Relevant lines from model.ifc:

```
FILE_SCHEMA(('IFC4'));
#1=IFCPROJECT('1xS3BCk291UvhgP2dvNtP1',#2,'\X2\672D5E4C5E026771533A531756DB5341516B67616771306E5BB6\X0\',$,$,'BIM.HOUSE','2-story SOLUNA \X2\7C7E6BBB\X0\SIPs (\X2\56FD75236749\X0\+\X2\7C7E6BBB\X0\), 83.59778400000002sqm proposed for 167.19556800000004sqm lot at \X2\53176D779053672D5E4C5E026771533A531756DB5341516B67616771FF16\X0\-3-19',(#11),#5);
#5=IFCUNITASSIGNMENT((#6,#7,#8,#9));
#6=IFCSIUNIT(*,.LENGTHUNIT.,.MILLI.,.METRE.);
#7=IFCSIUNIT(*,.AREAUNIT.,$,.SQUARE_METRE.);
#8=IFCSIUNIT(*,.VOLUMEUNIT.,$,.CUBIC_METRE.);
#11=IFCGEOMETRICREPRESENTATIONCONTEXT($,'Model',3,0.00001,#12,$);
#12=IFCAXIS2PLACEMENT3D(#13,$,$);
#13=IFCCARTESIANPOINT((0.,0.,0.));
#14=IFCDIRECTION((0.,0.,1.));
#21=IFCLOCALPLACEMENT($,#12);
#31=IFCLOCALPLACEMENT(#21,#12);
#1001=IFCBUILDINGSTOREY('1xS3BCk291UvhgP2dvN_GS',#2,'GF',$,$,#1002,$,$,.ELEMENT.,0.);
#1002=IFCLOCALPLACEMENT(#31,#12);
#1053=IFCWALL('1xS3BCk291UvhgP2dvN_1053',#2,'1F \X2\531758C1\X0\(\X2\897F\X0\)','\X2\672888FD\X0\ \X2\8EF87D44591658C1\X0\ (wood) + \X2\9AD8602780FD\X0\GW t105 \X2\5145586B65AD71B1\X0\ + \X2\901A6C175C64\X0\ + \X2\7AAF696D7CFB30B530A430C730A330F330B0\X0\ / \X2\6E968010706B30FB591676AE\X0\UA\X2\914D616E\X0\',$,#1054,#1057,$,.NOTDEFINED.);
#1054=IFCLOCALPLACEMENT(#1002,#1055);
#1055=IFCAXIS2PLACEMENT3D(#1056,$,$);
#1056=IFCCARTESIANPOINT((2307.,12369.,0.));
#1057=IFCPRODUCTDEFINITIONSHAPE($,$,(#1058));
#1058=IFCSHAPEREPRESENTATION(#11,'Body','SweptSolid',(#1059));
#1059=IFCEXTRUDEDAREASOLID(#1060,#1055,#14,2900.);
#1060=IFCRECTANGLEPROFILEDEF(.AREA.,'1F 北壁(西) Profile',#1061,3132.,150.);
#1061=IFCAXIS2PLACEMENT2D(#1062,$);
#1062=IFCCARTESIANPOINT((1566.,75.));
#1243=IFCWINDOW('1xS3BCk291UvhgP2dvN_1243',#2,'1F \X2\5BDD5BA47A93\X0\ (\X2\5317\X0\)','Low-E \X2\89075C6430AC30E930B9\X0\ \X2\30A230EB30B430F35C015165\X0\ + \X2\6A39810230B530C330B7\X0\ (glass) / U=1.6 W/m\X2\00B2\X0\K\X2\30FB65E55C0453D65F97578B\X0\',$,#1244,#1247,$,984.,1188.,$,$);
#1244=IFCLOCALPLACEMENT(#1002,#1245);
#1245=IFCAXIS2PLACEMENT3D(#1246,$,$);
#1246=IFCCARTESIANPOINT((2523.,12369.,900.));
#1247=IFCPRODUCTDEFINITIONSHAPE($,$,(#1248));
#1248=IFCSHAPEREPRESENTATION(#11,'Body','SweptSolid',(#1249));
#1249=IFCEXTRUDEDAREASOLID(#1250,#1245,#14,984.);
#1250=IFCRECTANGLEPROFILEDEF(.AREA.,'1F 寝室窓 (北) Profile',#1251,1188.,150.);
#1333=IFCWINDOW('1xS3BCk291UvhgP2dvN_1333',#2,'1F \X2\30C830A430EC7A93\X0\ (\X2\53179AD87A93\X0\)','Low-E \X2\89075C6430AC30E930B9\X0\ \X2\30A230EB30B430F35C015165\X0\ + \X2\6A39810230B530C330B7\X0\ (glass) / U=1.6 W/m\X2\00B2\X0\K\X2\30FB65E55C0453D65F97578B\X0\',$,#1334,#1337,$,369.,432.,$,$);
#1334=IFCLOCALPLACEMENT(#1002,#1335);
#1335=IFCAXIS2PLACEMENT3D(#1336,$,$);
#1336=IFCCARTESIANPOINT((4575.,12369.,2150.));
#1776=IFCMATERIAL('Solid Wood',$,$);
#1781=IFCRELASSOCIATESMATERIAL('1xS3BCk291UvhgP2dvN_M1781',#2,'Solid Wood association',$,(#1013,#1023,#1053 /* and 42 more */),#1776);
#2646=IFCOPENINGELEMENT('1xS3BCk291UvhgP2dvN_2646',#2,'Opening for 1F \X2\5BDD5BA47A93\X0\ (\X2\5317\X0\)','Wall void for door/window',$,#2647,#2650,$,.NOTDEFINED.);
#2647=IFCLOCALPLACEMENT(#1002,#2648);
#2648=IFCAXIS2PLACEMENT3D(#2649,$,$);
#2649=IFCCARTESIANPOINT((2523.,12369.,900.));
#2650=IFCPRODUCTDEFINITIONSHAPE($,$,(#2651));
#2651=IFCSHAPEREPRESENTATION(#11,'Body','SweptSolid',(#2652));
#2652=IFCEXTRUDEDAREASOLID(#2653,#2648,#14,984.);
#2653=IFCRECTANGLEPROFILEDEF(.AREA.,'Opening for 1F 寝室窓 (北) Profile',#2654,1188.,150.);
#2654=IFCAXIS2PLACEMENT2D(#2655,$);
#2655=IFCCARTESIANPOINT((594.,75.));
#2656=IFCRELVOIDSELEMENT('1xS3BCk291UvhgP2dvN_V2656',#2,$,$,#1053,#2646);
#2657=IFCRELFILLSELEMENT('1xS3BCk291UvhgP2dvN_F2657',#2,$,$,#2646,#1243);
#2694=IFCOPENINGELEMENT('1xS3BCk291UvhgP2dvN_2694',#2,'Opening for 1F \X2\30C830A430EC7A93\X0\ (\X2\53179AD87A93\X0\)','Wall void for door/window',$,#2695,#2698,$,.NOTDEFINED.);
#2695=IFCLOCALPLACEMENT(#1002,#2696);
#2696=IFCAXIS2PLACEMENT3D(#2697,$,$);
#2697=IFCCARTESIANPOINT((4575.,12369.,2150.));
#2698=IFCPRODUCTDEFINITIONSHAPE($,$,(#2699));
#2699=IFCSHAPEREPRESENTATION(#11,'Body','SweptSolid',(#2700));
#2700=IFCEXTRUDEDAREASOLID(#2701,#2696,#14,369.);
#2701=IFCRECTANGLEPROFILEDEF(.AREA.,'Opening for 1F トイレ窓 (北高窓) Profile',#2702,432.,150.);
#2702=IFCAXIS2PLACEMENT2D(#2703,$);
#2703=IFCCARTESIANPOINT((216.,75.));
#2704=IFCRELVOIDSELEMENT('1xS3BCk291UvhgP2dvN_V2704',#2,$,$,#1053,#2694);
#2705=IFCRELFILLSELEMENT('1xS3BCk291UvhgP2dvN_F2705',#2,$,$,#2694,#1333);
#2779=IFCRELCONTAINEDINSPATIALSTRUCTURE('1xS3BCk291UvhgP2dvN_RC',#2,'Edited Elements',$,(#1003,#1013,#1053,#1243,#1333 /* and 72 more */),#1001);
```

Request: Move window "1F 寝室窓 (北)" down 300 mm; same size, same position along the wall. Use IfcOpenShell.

```python
import numpy as np
import ifcopenshell
import ifcopenshell.api.geometry
import ifcopenshell.util.placement
import ifcopenshell.util.unit

model = ifcopenshell.open("model.ifc")
unit_scale = ifcopenshell.util.unit.calculate_unit_scale(model)

window = model.by_guid("1xS3BCk291UvhgP2dvN_1243")
opening = window.FillsVoids[0].RelatingOpeningElement
dz = -300.0

shift = np.array([0.0, 0.0, dz])
# The window is not placed relative to its opening, so move both.
for product in (opening, window):
    matrix = ifcopenshell.util.placement.get_local_placement(product.ObjectPlacement)
    matrix[:3, 3] += shift
    ifcopenshell.api.geometry.edit_object_placement(model, product=product, matrix=matrix, is_si=False)

print(f"moved by {dz * unit_scale:+.3f} m")

model.write("model_updated.ifc")
```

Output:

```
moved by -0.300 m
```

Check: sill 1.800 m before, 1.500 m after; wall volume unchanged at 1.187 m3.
